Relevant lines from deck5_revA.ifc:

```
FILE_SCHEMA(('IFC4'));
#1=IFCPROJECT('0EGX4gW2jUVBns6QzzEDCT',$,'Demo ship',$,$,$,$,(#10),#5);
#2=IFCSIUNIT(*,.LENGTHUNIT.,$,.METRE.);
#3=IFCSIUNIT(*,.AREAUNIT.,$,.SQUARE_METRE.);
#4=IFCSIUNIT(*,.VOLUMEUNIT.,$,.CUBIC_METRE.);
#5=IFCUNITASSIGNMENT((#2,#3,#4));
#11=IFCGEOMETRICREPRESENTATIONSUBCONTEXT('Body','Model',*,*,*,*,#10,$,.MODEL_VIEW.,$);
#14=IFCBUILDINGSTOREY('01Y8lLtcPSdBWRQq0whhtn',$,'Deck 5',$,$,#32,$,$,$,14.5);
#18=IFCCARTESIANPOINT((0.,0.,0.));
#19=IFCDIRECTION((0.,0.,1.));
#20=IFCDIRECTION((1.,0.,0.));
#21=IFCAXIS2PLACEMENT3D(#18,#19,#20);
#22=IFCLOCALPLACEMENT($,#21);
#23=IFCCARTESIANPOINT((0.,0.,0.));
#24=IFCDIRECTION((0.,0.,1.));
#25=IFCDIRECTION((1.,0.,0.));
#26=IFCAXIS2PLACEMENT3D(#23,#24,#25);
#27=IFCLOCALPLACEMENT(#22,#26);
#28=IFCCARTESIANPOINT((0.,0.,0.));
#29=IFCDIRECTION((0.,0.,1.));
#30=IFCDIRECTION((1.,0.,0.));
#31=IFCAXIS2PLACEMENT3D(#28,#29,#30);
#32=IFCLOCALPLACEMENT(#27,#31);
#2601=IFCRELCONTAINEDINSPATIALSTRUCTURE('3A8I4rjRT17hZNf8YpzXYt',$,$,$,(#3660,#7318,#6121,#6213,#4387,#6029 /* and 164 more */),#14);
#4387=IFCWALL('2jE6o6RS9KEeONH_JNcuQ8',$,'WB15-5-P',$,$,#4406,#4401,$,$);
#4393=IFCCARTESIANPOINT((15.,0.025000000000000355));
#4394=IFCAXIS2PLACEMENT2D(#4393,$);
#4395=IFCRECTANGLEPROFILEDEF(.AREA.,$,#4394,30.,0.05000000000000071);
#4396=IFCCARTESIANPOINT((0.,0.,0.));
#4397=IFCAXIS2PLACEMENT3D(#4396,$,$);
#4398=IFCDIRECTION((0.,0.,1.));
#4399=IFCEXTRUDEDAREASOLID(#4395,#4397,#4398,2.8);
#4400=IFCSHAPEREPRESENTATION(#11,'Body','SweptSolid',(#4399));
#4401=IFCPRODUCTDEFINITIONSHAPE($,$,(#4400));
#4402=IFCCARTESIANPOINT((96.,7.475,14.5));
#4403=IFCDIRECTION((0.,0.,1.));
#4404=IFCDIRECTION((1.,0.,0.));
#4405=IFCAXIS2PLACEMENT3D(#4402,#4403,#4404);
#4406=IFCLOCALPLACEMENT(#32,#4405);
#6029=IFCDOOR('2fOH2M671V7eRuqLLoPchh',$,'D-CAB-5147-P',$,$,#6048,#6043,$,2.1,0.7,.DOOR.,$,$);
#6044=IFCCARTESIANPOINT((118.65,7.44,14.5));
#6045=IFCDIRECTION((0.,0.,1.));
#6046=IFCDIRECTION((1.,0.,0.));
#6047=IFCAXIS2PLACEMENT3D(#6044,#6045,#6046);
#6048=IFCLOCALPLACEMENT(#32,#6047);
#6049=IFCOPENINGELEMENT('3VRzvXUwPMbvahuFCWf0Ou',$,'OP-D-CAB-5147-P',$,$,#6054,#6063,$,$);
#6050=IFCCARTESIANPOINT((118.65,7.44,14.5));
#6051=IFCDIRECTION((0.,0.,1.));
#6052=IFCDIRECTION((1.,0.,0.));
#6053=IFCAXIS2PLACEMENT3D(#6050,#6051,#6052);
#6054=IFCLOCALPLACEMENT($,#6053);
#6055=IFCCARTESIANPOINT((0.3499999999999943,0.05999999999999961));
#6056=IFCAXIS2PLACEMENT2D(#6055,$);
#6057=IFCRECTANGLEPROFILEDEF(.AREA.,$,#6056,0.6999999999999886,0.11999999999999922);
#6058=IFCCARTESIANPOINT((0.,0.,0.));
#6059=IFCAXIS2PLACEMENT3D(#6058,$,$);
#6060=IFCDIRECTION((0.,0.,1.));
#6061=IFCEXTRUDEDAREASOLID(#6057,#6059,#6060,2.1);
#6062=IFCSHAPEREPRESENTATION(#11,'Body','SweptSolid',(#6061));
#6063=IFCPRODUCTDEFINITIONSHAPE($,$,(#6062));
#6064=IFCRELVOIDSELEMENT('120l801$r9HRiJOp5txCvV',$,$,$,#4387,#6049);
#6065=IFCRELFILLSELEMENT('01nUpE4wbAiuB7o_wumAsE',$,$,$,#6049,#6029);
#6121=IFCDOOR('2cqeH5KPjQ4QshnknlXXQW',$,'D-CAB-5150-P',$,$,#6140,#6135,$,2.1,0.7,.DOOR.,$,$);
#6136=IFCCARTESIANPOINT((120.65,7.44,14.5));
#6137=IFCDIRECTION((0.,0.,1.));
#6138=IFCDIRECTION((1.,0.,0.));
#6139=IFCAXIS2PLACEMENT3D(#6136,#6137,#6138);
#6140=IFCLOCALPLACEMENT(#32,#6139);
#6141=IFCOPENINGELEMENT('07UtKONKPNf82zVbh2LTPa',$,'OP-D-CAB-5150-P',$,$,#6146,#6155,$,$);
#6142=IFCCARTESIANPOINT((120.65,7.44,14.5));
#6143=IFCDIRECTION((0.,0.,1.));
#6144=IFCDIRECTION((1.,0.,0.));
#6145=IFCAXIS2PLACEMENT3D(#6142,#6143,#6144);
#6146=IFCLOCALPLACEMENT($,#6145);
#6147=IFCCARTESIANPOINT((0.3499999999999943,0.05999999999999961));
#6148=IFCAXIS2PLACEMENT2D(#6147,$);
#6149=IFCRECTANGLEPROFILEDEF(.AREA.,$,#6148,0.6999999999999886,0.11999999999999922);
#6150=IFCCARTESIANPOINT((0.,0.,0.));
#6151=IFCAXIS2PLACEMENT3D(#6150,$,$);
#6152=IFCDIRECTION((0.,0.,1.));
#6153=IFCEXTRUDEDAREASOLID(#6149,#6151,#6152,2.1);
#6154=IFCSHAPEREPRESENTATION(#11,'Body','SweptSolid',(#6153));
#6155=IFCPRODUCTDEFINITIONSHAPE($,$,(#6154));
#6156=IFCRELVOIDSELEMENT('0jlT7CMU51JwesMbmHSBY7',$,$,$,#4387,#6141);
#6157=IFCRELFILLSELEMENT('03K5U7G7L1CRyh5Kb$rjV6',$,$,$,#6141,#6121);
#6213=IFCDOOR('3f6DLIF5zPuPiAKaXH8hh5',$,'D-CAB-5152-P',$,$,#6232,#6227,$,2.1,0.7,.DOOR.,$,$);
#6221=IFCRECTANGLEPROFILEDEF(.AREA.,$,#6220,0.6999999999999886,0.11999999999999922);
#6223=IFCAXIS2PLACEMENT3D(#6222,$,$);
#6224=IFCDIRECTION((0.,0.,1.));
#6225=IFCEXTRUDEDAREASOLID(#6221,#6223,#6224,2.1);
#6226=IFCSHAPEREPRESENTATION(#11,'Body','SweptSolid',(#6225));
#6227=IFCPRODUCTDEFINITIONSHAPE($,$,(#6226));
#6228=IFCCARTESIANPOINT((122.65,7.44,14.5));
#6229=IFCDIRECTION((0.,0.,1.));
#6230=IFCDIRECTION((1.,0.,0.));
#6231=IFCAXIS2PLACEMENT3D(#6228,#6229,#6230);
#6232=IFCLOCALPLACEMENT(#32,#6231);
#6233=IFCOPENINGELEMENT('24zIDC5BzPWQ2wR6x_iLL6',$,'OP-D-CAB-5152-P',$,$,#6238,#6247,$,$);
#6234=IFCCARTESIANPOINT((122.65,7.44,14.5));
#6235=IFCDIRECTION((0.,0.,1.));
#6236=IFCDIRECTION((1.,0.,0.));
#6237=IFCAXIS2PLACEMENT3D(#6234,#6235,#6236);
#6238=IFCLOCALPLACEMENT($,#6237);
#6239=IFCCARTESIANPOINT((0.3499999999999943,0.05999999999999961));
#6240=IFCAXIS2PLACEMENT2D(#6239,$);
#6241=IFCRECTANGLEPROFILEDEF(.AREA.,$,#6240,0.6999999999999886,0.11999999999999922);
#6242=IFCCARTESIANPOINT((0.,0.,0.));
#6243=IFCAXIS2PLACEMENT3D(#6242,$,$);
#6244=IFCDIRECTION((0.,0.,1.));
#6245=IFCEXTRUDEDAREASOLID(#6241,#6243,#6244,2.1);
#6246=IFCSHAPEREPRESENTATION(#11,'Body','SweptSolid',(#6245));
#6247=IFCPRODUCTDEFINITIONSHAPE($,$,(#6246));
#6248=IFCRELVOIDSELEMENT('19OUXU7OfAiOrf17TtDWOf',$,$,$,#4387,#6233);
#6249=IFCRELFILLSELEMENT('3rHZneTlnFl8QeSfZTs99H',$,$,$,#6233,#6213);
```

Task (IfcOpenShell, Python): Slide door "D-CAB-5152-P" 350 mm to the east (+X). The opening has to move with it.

```python
import ifcopenshell
import ifcopenshell.api.geometry
import ifcopenshell.util.placement
import ifcopenshell.util.unit

model = ifcopenshell.open("deck5_revA.ifc")
unit_scale = ifcopenshell.util.unit.calculate_unit_scale(model)

door = model.by_guid("3f6DLIF5zPuPiAKaXH8hh5")
opening = door.FillsVoids[0].RelatingOpeningElement
wall = opening.VoidsElements[0].RelatingBuildingElement

wall_matrix = ifcopenshell.util.placement.get_local_placement(wall.ObjectPlacement)
shift = wall_matrix[:3, 0] * 0.35 / unit_scale
before = ifcopenshell.util.placement.get_local_placement(door.ObjectPlacement)[:3, 3].copy()

# The door is not placed relative to its opening, so move both.
for product in (opening, door):
    matrix = ifcopenshell.util.placement.get_local_placement(product.ObjectPlacement)
    matrix[:3, 3] += shift
    ifcopenshell.api.geometry.edit_object_placement(model, product=product, matrix=matrix, is_si=False)

after = ifcopenshell.util.placement.get_local_placement(door.ObjectPlacement)[:3, 3]
print("door moved by", (after - before).round(3) + 0.0)

model.write("deck5_revA_v2.ifc")
```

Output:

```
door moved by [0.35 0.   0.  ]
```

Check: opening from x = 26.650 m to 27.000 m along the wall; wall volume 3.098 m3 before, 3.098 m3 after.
